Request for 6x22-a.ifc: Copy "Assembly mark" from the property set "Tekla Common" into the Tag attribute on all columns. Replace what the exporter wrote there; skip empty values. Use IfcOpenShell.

First a look at what the model holds.

```python
import ifcopenshell
import ifcopenshell.util.element

model = ifcopenshell.open("6x22-a.ifc")
print(model.schema)
columns = model.by_type("IfcColumn")
print(len(columns), "columns")
for e in columns[:8]:
    source = ifcopenshell.util.element.get_pset(e, "Tekla Common", "Assembly mark")
    target = e.Tag
    print(e.id(), repr(source), repr(target), sep=" | ")
```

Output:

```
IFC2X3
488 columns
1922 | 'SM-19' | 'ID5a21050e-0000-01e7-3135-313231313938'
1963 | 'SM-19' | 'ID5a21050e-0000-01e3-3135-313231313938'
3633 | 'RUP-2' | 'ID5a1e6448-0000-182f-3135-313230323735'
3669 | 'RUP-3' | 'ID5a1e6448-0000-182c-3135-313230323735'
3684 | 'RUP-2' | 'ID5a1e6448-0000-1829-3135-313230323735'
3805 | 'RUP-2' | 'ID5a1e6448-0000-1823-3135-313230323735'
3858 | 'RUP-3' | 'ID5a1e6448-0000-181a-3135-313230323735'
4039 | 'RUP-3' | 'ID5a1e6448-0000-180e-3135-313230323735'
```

```python
import ifcopenshell
import ifcopenshell.util.element

model = ifcopenshell.open("6x22-a.ifc")

count = 0
for e in model.by_type("IfcColumn"):
    value = ifcopenshell.util.element.get_pset(e, "Tekla Common", "Assembly mark")
    current = e.Tag
    if not value or not value.strip() or current == value:
        continue
    e.Tag = value
    count += 1

print(count, "columns updated")

model.write("6x22-a_rev.ifc")
```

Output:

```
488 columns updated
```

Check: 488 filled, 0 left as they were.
